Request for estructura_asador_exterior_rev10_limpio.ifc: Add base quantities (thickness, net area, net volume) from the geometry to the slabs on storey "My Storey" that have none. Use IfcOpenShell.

First a look at what the model holds.

```python
import ifcopenshell
import ifcopenshell.util.element
import ifcopenshell.util.unit

model = ifcopenshell.open("estructura_asador_exterior_rev10_limpio.ifc")
print(model.schema)
for unit_type in ("LENGTHUNIT", "AREAUNIT", "VOLUMEUNIT"):
    print(unit_type, ifcopenshell.util.unit.calculate_unit_scale(model, unit_type))
storey = next(s for s in model.by_type("IfcBuildingStorey") if s.Name == "My Storey")
slabs = [e for e in ifcopenshell.util.element.get_decomposition(storey) if e.is_a("IfcSlab")]
for e in sorted(slabs, key=lambda e: e.id()):
    print(e.id(), e.is_a(), e.Name, list(ifcopenshell.util.element.get_psets(e, qtos_only=True)), sep=" | ")
```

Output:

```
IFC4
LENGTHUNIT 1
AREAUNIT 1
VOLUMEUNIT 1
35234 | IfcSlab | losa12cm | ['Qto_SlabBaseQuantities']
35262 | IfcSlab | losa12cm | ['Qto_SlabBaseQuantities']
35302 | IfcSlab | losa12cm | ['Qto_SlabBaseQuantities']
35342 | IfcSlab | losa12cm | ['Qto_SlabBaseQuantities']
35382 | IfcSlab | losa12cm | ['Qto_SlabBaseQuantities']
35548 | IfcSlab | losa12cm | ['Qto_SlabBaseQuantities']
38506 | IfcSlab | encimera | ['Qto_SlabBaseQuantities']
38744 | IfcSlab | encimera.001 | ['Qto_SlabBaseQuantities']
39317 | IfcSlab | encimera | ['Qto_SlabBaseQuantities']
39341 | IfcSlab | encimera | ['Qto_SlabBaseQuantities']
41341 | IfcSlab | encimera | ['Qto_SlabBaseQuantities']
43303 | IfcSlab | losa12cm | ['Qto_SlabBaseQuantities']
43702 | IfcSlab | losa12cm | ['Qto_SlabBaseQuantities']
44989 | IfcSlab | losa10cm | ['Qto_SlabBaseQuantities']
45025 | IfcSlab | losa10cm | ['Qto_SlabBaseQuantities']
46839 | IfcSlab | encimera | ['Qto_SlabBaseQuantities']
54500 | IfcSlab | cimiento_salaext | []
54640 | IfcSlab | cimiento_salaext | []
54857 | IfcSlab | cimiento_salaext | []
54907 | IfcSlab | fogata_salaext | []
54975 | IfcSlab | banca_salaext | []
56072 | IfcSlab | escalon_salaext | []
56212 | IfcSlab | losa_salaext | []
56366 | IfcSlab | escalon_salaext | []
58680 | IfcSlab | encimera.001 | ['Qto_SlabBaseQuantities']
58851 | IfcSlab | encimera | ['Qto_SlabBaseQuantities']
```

```python
import ifcopenshell
import ifcopenshell.api.pset
import ifcopenshell.geom
import ifcopenshell.util.element
import ifcopenshell.util.shape
import ifcopenshell.util.unit

model = ifcopenshell.open("estructura_asador_exterior_rev10_limpio.ifc")
unit_scale = ifcopenshell.util.unit.calculate_unit_scale(model)
area_scale = ifcopenshell.util.unit.calculate_unit_scale(model, "AREAUNIT")
volume_scale = ifcopenshell.util.unit.calculate_unit_scale(model, "VOLUMEUNIT")
settings = ifcopenshell.geom.settings()

storey = next(s for s in model.by_type("IfcBuildingStorey") if s.Name == "My Storey")
slabs = [e for e in ifcopenshell.util.element.get_decomposition(storey) if e.is_a("IfcSlab")]

for e in sorted(slabs, key=lambda e: e.id()):
    if ifcopenshell.util.element.get_psets(e, qtos_only=True, should_inherit=False):
        continue
    # Geometry comes back in metres, in the element's own axes.
    shape = ifcopenshell.geom.create_shape(settings, e)
    values = {
        "Width": ifcopenshell.util.shape.get_z(shape.geometry) / unit_scale,
        "NetArea": ifcopenshell.util.shape.get_footprint_area(shape.geometry) / area_scale,
        "NetVolume": ifcopenshell.util.shape.get_volume(shape.geometry) / volume_scale,
    }
    qto = ifcopenshell.api.pset.add_qto(model, product=e, name="Qto_SlabBaseQuantities")
    ifcopenshell.api.pset.edit_qto(model, qto=qto, properties=values)
    print(e.id(), {k: round(v, 3) for k, v in values.items()})

model.write("estructura_asador_exterior_rev10_limpio_v2.ifc")
```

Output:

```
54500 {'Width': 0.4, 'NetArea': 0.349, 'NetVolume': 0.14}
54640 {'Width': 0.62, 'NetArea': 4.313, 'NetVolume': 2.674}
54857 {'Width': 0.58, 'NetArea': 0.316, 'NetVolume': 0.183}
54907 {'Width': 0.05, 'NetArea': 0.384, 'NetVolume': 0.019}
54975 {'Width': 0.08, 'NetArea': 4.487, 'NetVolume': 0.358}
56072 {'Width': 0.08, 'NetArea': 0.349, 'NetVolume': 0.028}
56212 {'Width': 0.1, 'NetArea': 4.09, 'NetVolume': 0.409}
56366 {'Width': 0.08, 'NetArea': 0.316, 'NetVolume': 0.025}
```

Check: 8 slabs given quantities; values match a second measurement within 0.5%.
